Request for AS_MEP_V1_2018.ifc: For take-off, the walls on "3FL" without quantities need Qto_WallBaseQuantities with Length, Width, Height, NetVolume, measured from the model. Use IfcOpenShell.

First a look at what the model holds.

```python
import ifcopenshell
import ifcopenshell.util.element
import ifcopenshell.util.unit

model = ifcopenshell.open("AS_MEP_V1_2018.ifc")
print(model.schema)
for unit_type in ("LENGTHUNIT", "AREAUNIT", "VOLUMEUNIT"):
    print(unit_type, ifcopenshell.util.unit.calculate_unit_scale(model, unit_type))
storey = next(s for s in model.by_type("IfcBuildingStorey") if s.Name == "3FL")
walls = [e for e in ifcopenshell.util.element.get_decomposition(storey) if e.is_a("IfcWall")]
for e in sorted(walls, key=lambda e: e.id()):
    print(e.id(), e.is_a(), e.Name, list(ifcopenshell.util.element.get_psets(e, qtos_only=True)), sep=" | ")
```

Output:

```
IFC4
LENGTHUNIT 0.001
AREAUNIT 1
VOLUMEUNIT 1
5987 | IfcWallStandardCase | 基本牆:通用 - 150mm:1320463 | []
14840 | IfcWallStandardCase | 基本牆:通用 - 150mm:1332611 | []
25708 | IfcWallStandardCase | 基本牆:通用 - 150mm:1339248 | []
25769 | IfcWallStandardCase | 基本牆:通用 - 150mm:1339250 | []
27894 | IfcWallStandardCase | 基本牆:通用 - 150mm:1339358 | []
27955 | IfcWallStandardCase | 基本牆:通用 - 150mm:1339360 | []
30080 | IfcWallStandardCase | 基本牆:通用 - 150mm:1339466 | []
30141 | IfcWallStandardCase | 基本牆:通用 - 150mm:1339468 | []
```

```python
import ifcopenshell
import ifcopenshell.api.pset
import ifcopenshell.geom
import ifcopenshell.util.element
import ifcopenshell.util.shape
import ifcopenshell.util.unit

model = ifcopenshell.open("AS_MEP_V1_2018.ifc")
unit_scale = ifcopenshell.util.unit.calculate_unit_scale(model)
volume_scale = ifcopenshell.util.unit.calculate_unit_scale(model, "VOLUMEUNIT")
settings = ifcopenshell.geom.settings()

storey = next(s for s in model.by_type("IfcBuildingStorey") if s.Name == "3FL")
walls = [e for e in ifcopenshell.util.element.get_decomposition(storey) if e.is_a("IfcWall")]

for e in sorted(walls, key=lambda e: e.id()):
    if ifcopenshell.util.element.get_psets(e, qtos_only=True, should_inherit=False):
        continue
    # Geometry comes back in metres, in the element's own axes.
    shape = ifcopenshell.geom.create_shape(settings, e)
    values = {
        "Length": ifcopenshell.util.shape.get_x(shape.geometry) / unit_scale,
        "Width": ifcopenshell.util.shape.get_y(shape.geometry) / unit_scale,
        "Height": ifcopenshell.util.shape.get_z(shape.geometry) / unit_scale,
        "NetVolume": ifcopenshell.util.shape.get_volume(shape.geometry) / volume_scale,
    }
    qto = ifcopenshell.api.pset.add_qto(model, product=e, name="Qto_WallBaseQuantities")
    ifcopenshell.api.pset.edit_qto(model, qto=qto, properties=values)
    print(e.id(), {k: round(v, 3) for k, v in values.items()})

model.write("AS_MEP_V1_2018_rev.ifc")
```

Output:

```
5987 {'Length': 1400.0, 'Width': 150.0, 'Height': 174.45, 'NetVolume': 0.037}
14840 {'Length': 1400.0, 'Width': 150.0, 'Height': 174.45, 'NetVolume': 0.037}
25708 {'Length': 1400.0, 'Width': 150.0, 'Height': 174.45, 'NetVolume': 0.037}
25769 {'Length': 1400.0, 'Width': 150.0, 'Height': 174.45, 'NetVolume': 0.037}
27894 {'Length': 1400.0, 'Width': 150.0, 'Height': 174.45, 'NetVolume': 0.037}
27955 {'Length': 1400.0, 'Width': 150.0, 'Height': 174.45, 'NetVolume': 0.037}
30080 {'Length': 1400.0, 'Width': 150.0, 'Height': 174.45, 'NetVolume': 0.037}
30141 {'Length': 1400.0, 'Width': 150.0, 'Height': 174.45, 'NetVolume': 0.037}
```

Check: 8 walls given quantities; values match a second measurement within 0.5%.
